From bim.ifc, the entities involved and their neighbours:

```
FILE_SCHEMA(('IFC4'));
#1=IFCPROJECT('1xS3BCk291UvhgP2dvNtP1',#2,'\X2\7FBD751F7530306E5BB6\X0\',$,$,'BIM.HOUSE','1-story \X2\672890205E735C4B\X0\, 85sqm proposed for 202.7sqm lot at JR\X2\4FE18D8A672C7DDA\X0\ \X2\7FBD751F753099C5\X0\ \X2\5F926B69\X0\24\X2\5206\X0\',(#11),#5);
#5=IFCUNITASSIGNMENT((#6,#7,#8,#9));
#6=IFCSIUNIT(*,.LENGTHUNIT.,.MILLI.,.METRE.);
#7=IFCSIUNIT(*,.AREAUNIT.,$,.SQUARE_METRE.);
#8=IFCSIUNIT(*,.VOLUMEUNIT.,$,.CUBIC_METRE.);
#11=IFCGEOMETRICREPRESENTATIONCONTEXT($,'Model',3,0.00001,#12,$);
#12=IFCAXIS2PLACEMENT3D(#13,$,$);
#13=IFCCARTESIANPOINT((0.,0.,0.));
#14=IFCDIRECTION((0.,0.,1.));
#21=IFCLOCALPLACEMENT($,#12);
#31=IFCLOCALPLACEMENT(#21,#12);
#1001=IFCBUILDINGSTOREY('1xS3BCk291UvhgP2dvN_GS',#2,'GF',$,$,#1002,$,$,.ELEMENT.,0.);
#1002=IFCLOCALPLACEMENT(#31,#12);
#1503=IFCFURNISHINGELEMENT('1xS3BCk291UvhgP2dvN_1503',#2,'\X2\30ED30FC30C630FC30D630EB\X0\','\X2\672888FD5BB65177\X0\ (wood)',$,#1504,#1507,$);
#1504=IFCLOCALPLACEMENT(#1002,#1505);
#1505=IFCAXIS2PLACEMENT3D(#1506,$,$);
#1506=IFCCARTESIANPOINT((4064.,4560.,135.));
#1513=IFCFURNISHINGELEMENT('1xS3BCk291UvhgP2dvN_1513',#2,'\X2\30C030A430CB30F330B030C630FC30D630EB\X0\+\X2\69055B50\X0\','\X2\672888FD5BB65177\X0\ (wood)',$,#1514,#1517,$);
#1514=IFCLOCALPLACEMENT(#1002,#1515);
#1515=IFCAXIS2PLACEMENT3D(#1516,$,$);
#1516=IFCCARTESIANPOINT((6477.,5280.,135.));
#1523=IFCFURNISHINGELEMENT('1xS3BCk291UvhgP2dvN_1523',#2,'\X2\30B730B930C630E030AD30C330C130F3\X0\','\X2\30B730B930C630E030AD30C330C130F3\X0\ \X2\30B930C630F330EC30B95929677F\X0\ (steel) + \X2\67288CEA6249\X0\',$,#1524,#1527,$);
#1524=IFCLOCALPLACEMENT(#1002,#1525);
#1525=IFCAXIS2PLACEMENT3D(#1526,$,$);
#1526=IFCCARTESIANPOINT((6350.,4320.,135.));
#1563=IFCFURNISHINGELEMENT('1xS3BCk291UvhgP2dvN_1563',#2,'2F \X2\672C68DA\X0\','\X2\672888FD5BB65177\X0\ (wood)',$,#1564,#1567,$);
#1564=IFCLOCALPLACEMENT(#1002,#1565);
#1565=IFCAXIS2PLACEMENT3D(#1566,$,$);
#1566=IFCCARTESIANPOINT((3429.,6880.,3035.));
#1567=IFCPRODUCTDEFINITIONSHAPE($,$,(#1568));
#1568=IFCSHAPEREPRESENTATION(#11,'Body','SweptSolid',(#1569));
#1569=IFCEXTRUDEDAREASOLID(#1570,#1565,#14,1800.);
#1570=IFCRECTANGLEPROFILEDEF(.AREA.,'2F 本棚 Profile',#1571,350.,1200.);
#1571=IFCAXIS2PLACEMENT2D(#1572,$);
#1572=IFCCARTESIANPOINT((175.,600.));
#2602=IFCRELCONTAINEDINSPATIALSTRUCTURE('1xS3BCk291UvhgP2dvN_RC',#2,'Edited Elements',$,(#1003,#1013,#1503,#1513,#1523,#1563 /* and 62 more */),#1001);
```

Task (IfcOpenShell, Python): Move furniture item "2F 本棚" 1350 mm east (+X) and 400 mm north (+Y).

```python
import ifcopenshell
import ifcopenshell.api.geometry
import ifcopenshell.util.placement
import ifcopenshell.util.unit

model = ifcopenshell.open("bim.ifc")
unit_scale = ifcopenshell.util.unit.calculate_unit_scale(model)

item = model.by_guid("1xS3BCk291UvhgP2dvN_1563")
matrix = ifcopenshell.util.placement.get_local_placement(item.ObjectPlacement)
matrix[0, 3] += 1.35 / unit_scale
matrix[1, 3] += 0.4 / unit_scale
ifcopenshell.api.geometry.edit_object_placement(model, product=item, matrix=matrix, is_si=False)

print(ifcopenshell.util.placement.get_local_placement(item.ObjectPlacement).round(3) + 0.0)

model.write("bim_edited.ifc")
```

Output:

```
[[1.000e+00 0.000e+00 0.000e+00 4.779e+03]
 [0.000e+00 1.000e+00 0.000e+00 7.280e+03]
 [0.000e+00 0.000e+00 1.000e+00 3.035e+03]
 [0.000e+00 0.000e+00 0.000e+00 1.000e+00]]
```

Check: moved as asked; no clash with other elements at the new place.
